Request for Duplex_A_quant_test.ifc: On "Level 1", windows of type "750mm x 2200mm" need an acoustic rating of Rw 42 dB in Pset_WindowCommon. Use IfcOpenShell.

First a look at what the model holds.

```python
import ifcopenshell
import ifcopenshell.util.element

model = ifcopenshell.open("Duplex_A_quant_test.ifc")
print(model.schema)
storey = next(s for s in model.by_type("IfcBuildingStorey") if s.Name == "Level 1")
windows = [e for e in ifcopenshell.util.element.get_decomposition(storey) if e.is_a("IfcWindow")]
seen = {}
for e in windows:
    element_type = ifcopenshell.util.element.get_type(e)
    key = (element_type.Name if element_type != e and element_type else None, ifcopenshell.util.element.get_pset(e, "Pset_WindowCommon", "AcousticRating"))
    seen[key] = seen.get(key, 0) + 1
for (name, value), count in sorted(seen.items(), key=str):
    print(count, "x", name, "|", value)
```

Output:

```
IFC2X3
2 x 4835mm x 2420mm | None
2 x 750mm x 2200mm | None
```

```python
import ifcopenshell
import ifcopenshell.api.pset
import ifcopenshell.util.element

model = ifcopenshell.open("Duplex_A_quant_test.ifc")

storey = next(s for s in model.by_type("IfcBuildingStorey") if s.Name == "Level 1")
windows = [e for e in ifcopenshell.util.element.get_decomposition(storey) if e.is_a("IfcWindow")]

count = 0
for e in windows:
    element_type = ifcopenshell.util.element.get_type(e)
    if element_type in (None, e) or element_type.Name != "750mm x 2200mm":
        continue
    # add_pset returns the element's existing set when there is one.
    pset = ifcopenshell.api.pset.add_pset(model, product=e, name="Pset_WindowCommon")
    ifcopenshell.api.pset.edit_pset(model, pset=pset, properties={"AcousticRating": "Rw 42 dB"})
    count += 1

print(count, "windows updated")

model.write("Duplex_A_quant_test_edited.ifc")
```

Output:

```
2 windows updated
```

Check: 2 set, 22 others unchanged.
